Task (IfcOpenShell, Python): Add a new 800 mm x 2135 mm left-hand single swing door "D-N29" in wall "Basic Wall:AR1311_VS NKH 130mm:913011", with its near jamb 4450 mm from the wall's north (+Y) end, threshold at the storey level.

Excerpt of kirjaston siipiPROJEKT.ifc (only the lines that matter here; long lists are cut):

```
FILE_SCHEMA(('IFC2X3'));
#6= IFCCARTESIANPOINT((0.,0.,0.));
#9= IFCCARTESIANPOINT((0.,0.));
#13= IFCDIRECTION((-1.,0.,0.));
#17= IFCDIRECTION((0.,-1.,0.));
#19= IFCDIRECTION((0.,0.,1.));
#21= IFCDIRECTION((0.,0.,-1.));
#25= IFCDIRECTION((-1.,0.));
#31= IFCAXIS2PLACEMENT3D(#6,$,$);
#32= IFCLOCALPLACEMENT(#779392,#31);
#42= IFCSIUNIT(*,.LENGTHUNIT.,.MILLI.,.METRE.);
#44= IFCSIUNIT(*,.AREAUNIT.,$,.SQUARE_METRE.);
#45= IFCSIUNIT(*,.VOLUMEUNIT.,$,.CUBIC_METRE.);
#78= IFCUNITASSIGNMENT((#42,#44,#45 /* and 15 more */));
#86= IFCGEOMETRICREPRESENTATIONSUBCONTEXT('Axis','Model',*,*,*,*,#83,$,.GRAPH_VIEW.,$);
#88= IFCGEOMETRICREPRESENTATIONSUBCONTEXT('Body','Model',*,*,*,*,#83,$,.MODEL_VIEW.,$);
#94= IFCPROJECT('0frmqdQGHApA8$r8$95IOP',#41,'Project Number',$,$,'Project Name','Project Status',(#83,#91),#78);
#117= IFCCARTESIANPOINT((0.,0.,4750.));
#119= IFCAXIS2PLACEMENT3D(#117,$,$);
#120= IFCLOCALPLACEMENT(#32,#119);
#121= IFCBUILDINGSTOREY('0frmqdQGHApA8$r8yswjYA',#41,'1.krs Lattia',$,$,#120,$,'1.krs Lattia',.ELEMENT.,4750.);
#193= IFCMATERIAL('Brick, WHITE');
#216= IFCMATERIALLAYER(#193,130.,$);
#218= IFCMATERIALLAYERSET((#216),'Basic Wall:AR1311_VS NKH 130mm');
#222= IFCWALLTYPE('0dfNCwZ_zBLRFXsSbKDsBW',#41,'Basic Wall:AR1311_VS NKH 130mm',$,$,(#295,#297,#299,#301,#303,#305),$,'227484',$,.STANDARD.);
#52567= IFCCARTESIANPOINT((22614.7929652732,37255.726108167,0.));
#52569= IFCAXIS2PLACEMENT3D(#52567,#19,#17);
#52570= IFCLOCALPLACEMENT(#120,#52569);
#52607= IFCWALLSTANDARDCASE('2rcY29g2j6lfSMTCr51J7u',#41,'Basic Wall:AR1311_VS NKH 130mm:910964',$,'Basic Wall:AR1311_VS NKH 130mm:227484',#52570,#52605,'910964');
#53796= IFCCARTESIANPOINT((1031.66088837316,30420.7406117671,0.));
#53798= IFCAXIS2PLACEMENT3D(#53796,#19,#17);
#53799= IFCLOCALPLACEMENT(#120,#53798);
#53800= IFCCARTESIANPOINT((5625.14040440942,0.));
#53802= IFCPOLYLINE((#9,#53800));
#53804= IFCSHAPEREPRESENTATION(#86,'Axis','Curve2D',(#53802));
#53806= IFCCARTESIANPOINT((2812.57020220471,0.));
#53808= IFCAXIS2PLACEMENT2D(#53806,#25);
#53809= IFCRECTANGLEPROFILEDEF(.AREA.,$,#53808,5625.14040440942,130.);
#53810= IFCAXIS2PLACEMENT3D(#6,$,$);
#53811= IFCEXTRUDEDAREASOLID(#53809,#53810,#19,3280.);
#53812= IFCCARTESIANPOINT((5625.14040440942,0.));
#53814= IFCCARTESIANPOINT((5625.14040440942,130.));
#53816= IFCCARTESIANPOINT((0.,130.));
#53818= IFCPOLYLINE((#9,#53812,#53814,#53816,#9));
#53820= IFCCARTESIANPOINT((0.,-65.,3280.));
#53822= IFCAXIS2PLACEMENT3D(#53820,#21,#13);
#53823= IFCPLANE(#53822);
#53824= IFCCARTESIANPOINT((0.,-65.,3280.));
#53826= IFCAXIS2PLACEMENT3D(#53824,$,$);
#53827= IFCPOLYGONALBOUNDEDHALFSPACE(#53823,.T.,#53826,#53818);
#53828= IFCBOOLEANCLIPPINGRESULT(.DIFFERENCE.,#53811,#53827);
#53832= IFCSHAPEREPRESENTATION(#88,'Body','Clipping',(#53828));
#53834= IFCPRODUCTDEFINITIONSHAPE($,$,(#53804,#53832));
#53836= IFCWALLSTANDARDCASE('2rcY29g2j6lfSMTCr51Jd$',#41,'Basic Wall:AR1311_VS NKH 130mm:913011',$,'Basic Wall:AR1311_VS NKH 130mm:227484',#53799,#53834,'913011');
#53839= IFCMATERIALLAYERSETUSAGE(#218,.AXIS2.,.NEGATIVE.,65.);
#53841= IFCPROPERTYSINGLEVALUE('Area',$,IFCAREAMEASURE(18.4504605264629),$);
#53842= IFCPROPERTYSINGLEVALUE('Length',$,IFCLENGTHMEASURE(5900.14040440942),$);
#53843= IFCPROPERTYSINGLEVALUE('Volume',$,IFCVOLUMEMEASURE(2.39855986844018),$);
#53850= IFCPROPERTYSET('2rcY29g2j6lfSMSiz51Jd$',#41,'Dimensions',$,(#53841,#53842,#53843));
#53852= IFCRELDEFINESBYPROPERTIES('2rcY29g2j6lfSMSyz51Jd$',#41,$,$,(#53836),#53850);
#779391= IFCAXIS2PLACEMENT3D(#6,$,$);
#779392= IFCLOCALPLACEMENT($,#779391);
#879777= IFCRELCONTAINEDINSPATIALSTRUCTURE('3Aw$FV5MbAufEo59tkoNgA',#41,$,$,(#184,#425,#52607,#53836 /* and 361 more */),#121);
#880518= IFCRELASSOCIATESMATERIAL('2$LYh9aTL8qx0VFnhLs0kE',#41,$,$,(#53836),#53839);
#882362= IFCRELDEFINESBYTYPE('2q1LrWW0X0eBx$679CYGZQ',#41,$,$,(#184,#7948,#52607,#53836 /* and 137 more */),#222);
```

```python
import numpy as np
import ifcopenshell
import ifcopenshell.api.feature
import ifcopenshell.api.geometry
import ifcopenshell.api.pset
import ifcopenshell.api.root
import ifcopenshell.api.spatial
import ifcopenshell.api.type
import ifcopenshell.geom
import ifcopenshell.util.element
import ifcopenshell.util.placement
import ifcopenshell.util.representation
import ifcopenshell.util.shape
import ifcopenshell.util.unit

model = ifcopenshell.open("kirjaston siipiPROJEKT.ifc")
unit_scale = ifcopenshell.util.unit.calculate_unit_scale(model)
area_scale = ifcopenshell.util.unit.calculate_unit_scale(model, "AREAUNIT")
volume_scale = ifcopenshell.util.unit.calculate_unit_scale(model, "VOLUMEUNIT")
settings = ifcopenshell.geom.settings()


def volume(element):
    """Net volume in cubic metres, openings subtracted."""
    shape = ifcopenshell.geom.create_shape(settings, element)
    return ifcopenshell.util.shape.get_volume(shape.geometry)


wall = model.by_id(53836)
storey = ifcopenshell.util.element.get_container(wall, ifc_class="IfcBuildingStorey")
context = ifcopenshell.util.representation.get_context(model, "Model", "Body", "MODEL_VIEW")
before = volume(wall)

width, height, from_end, sill = 0.8, 2.135, 4.45, 0.0  # metres

# The wall runs along its own X axis, and the end named is its -X end.
wall_shape = ifcopenshell.geom.create_shape(settings, wall)
x, y, z = ifcopenshell.util.shape.get_vertices(wall_shape.geometry).T
start = x.min() + from_end
face, thickness = float(y.min()), float(y.max() - y.min())
wall_matrix = ifcopenshell.util.placement.get_local_placement(wall.ObjectPlacement)
level = ifcopenshell.util.placement.get_local_placement(storey.ObjectPlacement)[2, 3]


def in_wall(x, y):
    """Placement at x, y metres in the wall's axes, at sill height."""
    matrix = wall_matrix.copy()
    matrix[:, 3] = wall_matrix @ np.array([x / unit_scale, y / unit_scale, 0.0, 1.0])
    matrix[2, 3] = level + sill / unit_scale
    return matrix


# Opening: a box that overshoots both wall faces by 50 mm.
opening = ifcopenshell.api.root.create_entity(model, ifc_class="IfcOpeningElement")
box = ifcopenshell.api.geometry.add_wall_representation(
    model, context=context, length=width, height=height, thickness=thickness + 0.1
)
ifcopenshell.api.geometry.assign_representation(model, product=opening, representation=box)
ifcopenshell.api.geometry.edit_object_placement(model, product=opening, matrix=in_wall(start, face - 0.05), is_si=False)
ifcopenshell.api.feature.add_feature(model, feature=opening, element=wall)

door = ifcopenshell.api.root.create_entity(model, ifc_class="IfcDoor", name="D-N29")
door.OverallWidth, door.OverallHeight = width / unit_scale, height / unit_scale
body = ifcopenshell.api.geometry.add_door_representation(
    model,
    context=context,
    overall_width=door.OverallWidth,
    overall_height=door.OverallHeight,
    operation_type="SINGLE_SWING_LEFT",
    lining_properties={"LiningDepth": thickness / unit_scale, "ThresholdDepth": thickness / unit_scale},
)
ifcopenshell.api.geometry.assign_representation(model, product=door, representation=body)
ifcopenshell.api.spatial.assign_container(model, products=[door], relating_structure=storey)
fills = ifcopenshell.api.feature.add_filling(model, opening=opening, element=door)
fills.OwnerHistory = door.OwnerHistory  # required in IFC2X3

# IFC2X3 keeps the operation on the door style.
style = ifcopenshell.api.root.create_entity(model, ifc_class="IfcDoorStyle", name="D-N29")
style.OperationType, style.ConstructionType = "SINGLE_SWING_LEFT", "NOTDEFINED"
style.ParameterTakesPrecedence = style.Sizeable = False
ifcopenshell.api.type.assign_type(model, related_objects=[door], relating_type=style)

# The lining spans the wall, so the door starts at the wall face.
ifcopenshell.api.geometry.edit_object_placement(model, product=door, matrix=in_wall(start, face), is_si=False)

after = volume(wall)

# Update the wall's stored quantities.
pset = model.by_id(ifcopenshell.util.element.get_pset(wall, "Dimensions", should_inherit=False)["id"])
ifcopenshell.api.pset.edit_pset(model, pset=pset, properties={
    "Area": model.create_entity("IfcAreaMeasure", after / thickness / area_scale),
    "Volume": model.create_entity("IfcVolumeMeasure", after / volume_scale),
})

print(f"wall volume {before:.3f} -> {after:.3f} m3")

model.write("kirjaston siipiPROJEKT_v2.ifc")
```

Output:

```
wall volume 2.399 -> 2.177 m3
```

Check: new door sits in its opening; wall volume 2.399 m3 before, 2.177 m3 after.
